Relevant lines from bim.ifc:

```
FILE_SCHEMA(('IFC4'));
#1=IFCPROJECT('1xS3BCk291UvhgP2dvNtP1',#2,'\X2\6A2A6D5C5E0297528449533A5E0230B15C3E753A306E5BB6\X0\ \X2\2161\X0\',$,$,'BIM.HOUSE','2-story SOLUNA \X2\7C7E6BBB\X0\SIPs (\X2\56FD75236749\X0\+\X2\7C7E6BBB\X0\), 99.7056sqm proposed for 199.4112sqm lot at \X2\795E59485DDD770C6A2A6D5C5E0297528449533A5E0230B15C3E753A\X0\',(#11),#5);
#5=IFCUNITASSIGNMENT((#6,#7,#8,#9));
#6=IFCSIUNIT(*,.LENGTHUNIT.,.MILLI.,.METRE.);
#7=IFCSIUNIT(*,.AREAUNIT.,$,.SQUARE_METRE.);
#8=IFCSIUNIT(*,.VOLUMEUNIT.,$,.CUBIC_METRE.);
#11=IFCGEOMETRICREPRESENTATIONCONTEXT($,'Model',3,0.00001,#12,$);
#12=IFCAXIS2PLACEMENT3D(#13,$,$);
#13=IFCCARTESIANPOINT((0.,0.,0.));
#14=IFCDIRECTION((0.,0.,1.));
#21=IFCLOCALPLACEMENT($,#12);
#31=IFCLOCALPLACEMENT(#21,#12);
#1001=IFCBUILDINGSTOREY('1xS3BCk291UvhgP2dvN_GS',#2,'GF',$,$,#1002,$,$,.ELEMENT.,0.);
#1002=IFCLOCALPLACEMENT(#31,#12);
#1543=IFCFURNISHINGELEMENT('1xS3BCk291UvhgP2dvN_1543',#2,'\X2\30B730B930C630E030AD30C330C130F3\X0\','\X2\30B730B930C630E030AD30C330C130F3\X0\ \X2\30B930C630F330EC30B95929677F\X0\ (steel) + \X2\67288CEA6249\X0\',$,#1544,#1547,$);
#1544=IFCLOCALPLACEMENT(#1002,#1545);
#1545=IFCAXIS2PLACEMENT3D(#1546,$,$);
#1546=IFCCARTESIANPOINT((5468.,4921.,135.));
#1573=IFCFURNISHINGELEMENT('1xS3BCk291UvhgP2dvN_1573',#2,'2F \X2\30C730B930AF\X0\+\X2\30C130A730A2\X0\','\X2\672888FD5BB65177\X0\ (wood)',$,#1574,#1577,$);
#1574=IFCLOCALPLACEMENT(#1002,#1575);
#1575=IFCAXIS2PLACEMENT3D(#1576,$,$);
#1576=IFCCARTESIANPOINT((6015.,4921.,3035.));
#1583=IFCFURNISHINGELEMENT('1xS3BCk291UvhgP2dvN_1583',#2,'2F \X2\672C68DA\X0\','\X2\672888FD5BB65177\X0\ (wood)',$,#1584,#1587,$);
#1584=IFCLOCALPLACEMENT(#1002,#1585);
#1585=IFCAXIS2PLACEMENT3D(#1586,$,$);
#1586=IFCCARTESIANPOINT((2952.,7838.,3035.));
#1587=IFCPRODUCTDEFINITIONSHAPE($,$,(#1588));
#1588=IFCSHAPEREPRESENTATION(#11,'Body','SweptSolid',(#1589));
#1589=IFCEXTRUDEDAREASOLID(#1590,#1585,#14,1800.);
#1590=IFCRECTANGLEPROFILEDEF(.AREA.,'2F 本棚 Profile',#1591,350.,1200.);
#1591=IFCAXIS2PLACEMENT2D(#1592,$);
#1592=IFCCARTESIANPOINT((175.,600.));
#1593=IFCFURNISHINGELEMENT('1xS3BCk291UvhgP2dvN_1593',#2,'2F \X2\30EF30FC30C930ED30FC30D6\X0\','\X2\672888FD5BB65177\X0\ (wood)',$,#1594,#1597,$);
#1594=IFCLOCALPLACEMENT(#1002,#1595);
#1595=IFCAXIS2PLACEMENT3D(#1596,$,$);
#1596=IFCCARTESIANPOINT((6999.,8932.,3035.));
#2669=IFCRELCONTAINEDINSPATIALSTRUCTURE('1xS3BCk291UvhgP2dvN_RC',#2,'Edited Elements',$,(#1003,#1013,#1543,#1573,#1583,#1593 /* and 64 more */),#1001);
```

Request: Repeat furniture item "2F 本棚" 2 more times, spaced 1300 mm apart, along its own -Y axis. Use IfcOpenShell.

```python
import ifcopenshell
import ifcopenshell.api.geometry
import ifcopenshell.api.root
import ifcopenshell.util.element
import ifcopenshell.util.placement
import ifcopenshell.util.unit

model = ifcopenshell.open("bim.ifc")
unit_scale = ifcopenshell.util.unit.calculate_unit_scale(model)


def reuse_history(source, copy):
    """copy_class also copies each property set's owner history, people and application; keep the originals."""
    for rel in copy.IsDefinedBy:
        if rel.is_a("IfcRelDefinesByProperties") and (history := rel.RelatingPropertyDefinition.OwnerHistory):
            rel.RelatingPropertyDefinition.OwnerHistory = source.OwnerHistory
            ifcopenshell.util.element.remove_deep2(model, history)


source = model.by_guid("1xS3BCk291UvhgP2dvN_1583")
base = ifcopenshell.util.placement.get_local_placement(source.ObjectPlacement)
step = -base[:3, 1] * 1.3 / unit_scale

for i in range(1, 3):
    copy = ifcopenshell.api.root.copy_class(model, product=source)
    copy.Representation = ifcopenshell.util.element.copy_deep(
        model, source.Representation, exclude=["IfcGeometricRepresentationContext", "IfcRepresentationMap"]
    )
    reuse_history(source, copy)
    matrix = base.copy()
    matrix[:3, 3] += i * step
    print("added at", matrix[:3, 3].round(3) + 0.0)
    ifcopenshell.api.geometry.edit_object_placement(model, product=copy, matrix=matrix, is_si=False)

model.write("bim_updated.ifc")
```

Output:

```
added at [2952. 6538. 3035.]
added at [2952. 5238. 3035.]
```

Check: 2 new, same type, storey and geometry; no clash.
